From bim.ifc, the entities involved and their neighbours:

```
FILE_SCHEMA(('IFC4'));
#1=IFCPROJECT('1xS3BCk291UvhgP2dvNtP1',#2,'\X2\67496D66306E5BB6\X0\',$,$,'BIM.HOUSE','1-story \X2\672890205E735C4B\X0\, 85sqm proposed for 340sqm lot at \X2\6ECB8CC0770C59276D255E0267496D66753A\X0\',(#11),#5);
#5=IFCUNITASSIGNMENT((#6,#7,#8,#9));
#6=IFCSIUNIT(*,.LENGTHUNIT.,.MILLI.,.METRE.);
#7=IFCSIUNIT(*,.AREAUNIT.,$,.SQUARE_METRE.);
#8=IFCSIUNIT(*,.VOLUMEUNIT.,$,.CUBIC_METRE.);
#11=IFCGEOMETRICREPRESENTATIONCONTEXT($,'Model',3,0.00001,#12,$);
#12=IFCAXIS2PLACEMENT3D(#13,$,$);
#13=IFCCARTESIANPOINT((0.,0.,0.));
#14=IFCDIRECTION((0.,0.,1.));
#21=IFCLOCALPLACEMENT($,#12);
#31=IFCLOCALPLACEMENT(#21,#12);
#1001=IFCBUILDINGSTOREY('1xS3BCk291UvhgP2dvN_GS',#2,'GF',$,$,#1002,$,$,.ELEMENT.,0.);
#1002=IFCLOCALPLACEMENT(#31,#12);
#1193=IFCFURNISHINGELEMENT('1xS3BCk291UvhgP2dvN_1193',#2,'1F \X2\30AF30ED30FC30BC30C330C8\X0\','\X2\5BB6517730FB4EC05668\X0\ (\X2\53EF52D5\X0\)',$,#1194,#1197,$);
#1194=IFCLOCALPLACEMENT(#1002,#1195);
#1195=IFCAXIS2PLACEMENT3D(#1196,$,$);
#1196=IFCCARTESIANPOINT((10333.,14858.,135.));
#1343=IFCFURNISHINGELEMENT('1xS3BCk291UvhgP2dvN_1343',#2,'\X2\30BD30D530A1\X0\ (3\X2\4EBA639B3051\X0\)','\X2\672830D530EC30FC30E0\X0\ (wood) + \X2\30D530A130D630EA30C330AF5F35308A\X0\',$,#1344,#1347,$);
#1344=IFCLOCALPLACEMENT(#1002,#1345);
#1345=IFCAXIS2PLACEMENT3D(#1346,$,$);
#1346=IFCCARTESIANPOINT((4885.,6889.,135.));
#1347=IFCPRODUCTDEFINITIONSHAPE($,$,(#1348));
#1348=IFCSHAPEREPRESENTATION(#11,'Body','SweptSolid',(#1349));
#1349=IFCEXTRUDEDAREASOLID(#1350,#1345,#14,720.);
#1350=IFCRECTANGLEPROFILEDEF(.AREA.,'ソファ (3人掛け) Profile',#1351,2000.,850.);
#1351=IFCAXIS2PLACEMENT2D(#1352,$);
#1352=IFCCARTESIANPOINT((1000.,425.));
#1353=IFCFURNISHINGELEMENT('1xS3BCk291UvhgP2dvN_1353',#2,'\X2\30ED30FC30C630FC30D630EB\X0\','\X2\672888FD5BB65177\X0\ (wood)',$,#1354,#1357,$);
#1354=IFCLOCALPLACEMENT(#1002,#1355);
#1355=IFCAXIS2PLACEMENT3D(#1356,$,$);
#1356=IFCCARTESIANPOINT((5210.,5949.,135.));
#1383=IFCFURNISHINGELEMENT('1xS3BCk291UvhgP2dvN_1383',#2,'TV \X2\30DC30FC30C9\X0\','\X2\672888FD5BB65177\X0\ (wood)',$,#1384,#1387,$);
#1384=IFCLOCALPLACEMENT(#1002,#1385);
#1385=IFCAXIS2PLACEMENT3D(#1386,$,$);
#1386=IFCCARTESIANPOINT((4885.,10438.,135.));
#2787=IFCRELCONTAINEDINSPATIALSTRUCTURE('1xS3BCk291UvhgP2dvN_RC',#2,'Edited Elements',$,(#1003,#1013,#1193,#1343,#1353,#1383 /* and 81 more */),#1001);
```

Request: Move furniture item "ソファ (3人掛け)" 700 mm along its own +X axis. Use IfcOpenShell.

```python
import ifcopenshell
import ifcopenshell.api.geometry
import ifcopenshell.util.placement

model = ifcopenshell.open("bim.ifc")

item = model.by_id(1343)
matrix = ifcopenshell.util.placement.get_local_placement(item.ObjectPlacement)
matrix[:3, 3] += matrix[:3, 0] * 700.0
ifcopenshell.api.geometry.edit_object_placement(model, product=item, matrix=matrix, is_si=False)

print(ifcopenshell.util.placement.get_local_placement(item.ObjectPlacement).round(3) + 0.0)

model.write("bim_updated.ifc")
```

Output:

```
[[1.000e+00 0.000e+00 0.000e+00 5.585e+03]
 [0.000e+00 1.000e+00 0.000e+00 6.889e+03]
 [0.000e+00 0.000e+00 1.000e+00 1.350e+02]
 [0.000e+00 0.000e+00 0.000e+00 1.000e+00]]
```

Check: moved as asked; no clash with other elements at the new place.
